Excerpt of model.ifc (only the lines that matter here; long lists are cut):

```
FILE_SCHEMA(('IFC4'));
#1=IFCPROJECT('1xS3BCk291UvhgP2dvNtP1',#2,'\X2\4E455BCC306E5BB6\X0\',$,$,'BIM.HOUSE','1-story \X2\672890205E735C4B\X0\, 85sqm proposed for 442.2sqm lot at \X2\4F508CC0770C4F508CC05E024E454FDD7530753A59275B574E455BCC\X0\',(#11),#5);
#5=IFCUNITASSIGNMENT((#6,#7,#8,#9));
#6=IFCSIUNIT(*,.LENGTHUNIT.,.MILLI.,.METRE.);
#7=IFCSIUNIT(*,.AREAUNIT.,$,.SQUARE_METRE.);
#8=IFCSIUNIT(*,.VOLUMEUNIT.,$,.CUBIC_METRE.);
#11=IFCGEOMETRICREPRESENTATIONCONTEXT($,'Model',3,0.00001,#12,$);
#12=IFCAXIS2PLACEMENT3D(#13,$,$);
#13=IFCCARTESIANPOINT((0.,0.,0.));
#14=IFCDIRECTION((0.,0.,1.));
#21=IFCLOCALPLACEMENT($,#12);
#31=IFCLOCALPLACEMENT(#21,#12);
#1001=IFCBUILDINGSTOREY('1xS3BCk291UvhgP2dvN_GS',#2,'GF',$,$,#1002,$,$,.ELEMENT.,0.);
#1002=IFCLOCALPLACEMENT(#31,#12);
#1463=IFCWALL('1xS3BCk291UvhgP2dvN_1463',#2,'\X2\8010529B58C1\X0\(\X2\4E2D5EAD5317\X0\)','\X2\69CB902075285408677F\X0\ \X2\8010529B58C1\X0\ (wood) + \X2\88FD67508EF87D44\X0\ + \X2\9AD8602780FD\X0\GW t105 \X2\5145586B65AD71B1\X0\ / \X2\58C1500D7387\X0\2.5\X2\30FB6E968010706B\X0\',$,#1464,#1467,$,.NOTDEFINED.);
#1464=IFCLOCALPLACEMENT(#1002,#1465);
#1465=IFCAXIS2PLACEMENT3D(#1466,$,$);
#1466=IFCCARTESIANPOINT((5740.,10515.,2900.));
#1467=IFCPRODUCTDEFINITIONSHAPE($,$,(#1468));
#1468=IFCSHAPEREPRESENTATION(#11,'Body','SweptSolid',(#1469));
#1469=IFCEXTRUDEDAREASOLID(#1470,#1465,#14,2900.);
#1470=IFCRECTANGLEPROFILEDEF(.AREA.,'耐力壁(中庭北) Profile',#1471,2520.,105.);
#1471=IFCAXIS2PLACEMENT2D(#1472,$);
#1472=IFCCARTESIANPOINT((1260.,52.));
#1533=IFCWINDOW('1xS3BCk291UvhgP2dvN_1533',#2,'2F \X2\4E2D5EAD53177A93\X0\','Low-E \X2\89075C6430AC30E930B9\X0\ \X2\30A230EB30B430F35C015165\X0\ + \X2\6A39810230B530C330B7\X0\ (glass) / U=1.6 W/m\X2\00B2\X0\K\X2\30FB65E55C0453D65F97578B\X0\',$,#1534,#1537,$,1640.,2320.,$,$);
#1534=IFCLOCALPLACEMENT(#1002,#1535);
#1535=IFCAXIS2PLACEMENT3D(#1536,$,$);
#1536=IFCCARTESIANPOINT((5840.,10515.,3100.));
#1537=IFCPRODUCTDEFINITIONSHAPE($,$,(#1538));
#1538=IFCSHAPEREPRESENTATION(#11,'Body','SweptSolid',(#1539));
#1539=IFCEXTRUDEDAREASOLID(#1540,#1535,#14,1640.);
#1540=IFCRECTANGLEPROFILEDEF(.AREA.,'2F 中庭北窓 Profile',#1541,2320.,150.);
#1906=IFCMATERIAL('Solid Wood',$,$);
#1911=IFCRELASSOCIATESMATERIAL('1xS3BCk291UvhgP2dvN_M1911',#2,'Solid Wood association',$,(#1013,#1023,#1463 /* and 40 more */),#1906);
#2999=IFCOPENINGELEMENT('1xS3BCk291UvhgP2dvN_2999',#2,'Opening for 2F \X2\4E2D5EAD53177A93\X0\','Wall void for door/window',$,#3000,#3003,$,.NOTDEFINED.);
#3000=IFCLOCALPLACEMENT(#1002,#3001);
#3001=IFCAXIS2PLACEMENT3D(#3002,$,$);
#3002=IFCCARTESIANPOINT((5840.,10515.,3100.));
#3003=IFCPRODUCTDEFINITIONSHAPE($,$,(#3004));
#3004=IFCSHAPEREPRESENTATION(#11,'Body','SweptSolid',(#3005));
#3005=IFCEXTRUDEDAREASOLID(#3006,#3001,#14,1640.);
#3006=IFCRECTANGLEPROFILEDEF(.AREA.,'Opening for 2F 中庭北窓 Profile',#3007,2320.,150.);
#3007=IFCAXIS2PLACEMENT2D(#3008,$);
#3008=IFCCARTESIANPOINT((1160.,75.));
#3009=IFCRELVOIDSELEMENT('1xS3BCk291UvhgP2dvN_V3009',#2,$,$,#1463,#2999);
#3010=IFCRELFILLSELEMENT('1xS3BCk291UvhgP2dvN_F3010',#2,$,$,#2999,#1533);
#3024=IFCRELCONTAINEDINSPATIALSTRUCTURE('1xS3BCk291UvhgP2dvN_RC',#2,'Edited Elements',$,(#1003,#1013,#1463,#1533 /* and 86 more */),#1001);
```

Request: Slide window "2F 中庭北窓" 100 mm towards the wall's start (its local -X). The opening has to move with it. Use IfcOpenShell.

```python
import ifcopenshell
import ifcopenshell.api.geometry
import ifcopenshell.util.placement
import ifcopenshell.util.unit

model = ifcopenshell.open("model.ifc")
unit_scale = ifcopenshell.util.unit.calculate_unit_scale(model)

window = model.by_guid("1xS3BCk291UvhgP2dvN_1533")
opening = window.FillsVoids[0].RelatingOpeningElement
wall = opening.VoidsElements[0].RelatingBuildingElement

wall_matrix = ifcopenshell.util.placement.get_local_placement(wall.ObjectPlacement)
shift = wall_matrix[:3, 0] * -0.1 / unit_scale
before = ifcopenshell.util.placement.get_local_placement(window.ObjectPlacement)[:3, 3].copy()

# The window is not placed relative to its opening, so move both.
for product in (opening, window):
    matrix = ifcopenshell.util.placement.get_local_placement(product.ObjectPlacement)
    matrix[:3, 3] += shift
    ifcopenshell.api.geometry.edit_object_placement(model, product=product, matrix=matrix, is_si=False)

after = ifcopenshell.util.placement.get_local_placement(window.ObjectPlacement)[:3, 3]
print("window moved by", (after - before).round(3) + 0.0)

model.write("model_updated.ifc")
```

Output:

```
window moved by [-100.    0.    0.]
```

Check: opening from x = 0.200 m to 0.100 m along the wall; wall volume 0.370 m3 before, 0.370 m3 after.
